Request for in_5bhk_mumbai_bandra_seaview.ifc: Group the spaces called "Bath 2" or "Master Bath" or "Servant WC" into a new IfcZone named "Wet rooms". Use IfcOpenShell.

First a look at what the model holds.

```python
import ifcopenshell

model = ifcopenshell.open("in_5bhk_mumbai_bandra_seaview.ifc")
print(model.schema)
seen = {}
for space in model.by_type("IfcSpace"):
    seen[space.LongName] = seen.get(space.LongName, 0) + 1
for name, count in sorted(seen.items(), key=str):
    print(count, "x", name)
print("zones:", [z.Name for z in model.by_type("IfcZone")][:20])
```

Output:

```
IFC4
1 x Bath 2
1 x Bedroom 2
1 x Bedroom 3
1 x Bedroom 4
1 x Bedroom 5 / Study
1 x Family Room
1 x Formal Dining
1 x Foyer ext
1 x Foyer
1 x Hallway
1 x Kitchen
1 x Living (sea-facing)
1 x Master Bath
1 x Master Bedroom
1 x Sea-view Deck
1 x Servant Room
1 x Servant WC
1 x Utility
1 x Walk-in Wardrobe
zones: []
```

```python
import ifcopenshell
import ifcopenshell.api.group
import ifcopenshell.api.root

model = ifcopenshell.open("in_5bhk_mumbai_bandra_seaview.ifc")

names = {"Bath 2", "Master Bath", "Servant WC"}
spaces = [s for s in model.by_type("IfcSpace") if s.LongName in names]

zone = ifcopenshell.api.root.create_entity(model, ifc_class="IfcZone", name="Wet rooms")
ifcopenshell.api.group.assign_group(model, products=spaces, group=zone)
print(len(spaces), "spaces in", zone.Name)

model.write("in_5bhk_mumbai_bandra_seaview_updated.ifc")
```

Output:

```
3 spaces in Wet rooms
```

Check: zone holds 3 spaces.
